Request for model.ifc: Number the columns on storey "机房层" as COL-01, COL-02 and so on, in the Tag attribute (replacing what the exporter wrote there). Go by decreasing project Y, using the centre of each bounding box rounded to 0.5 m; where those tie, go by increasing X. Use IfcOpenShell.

First a look at what the model holds.

```python
import ifcopenshell
import ifcopenshell.util.element
import ifcopenshell.util.placement

model = ifcopenshell.open("model.ifc")
print(model.schema)
storey = next(s for s in model.by_type("IfcBuildingStorey") if s.Name == "机房层")
columns = [e for e in ifcopenshell.util.element.get_decomposition(storey) if e.is_a("IfcColumn")]
for e in sorted(columns, key=lambda e: e.id()):
    origin = ifcopenshell.util.placement.get_local_placement(e.ObjectPlacement)[:3, 3]
    print(e.id(), e.Tag, e.Name, origin.round(2) + 0.0, sep=" | ")
```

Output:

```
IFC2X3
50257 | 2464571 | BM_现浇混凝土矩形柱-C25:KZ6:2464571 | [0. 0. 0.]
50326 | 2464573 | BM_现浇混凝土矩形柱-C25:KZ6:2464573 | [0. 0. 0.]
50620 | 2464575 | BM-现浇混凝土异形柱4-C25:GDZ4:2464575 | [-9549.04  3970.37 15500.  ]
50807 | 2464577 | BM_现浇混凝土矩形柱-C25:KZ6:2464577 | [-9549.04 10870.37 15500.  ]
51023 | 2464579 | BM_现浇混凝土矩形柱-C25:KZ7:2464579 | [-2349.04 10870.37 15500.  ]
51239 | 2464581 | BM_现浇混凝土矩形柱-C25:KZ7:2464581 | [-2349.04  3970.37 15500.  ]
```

```python
import ifcopenshell
import ifcopenshell.geom
import ifcopenshell.util.element
import ifcopenshell.util.shape

model = ifcopenshell.open("model.ifc")
settings = ifcopenshell.geom.settings()
settings.set("use-world-coords", True)


def centre(element):
    shape = ifcopenshell.geom.create_shape(settings, element)
    return ifcopenshell.util.shape.get_bbox_centroid(shape.geometry)


storey = next(s for s in model.by_type("IfcBuildingStorey") if s.Name == "机房层")
columns = [e for e in ifcopenshell.util.element.get_decomposition(storey) if e.is_a("IfcColumn")]

# Insertion points can sit at a corner or the storey origin, so sort by the geometry (in metres).
centres = {e: centre(e) for e in columns}
columns.sort(key=lambda e: (-round(centres[e][1] / 0.5), centres[e][0]))

for i, e in enumerate(columns, start=1):
    number = f"COL-{i:02d}"
    e.Tag = number
    print(e.id(), number)

model.write("model_rev.ifc")
```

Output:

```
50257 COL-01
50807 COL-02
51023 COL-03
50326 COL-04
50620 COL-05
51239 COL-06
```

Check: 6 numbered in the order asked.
